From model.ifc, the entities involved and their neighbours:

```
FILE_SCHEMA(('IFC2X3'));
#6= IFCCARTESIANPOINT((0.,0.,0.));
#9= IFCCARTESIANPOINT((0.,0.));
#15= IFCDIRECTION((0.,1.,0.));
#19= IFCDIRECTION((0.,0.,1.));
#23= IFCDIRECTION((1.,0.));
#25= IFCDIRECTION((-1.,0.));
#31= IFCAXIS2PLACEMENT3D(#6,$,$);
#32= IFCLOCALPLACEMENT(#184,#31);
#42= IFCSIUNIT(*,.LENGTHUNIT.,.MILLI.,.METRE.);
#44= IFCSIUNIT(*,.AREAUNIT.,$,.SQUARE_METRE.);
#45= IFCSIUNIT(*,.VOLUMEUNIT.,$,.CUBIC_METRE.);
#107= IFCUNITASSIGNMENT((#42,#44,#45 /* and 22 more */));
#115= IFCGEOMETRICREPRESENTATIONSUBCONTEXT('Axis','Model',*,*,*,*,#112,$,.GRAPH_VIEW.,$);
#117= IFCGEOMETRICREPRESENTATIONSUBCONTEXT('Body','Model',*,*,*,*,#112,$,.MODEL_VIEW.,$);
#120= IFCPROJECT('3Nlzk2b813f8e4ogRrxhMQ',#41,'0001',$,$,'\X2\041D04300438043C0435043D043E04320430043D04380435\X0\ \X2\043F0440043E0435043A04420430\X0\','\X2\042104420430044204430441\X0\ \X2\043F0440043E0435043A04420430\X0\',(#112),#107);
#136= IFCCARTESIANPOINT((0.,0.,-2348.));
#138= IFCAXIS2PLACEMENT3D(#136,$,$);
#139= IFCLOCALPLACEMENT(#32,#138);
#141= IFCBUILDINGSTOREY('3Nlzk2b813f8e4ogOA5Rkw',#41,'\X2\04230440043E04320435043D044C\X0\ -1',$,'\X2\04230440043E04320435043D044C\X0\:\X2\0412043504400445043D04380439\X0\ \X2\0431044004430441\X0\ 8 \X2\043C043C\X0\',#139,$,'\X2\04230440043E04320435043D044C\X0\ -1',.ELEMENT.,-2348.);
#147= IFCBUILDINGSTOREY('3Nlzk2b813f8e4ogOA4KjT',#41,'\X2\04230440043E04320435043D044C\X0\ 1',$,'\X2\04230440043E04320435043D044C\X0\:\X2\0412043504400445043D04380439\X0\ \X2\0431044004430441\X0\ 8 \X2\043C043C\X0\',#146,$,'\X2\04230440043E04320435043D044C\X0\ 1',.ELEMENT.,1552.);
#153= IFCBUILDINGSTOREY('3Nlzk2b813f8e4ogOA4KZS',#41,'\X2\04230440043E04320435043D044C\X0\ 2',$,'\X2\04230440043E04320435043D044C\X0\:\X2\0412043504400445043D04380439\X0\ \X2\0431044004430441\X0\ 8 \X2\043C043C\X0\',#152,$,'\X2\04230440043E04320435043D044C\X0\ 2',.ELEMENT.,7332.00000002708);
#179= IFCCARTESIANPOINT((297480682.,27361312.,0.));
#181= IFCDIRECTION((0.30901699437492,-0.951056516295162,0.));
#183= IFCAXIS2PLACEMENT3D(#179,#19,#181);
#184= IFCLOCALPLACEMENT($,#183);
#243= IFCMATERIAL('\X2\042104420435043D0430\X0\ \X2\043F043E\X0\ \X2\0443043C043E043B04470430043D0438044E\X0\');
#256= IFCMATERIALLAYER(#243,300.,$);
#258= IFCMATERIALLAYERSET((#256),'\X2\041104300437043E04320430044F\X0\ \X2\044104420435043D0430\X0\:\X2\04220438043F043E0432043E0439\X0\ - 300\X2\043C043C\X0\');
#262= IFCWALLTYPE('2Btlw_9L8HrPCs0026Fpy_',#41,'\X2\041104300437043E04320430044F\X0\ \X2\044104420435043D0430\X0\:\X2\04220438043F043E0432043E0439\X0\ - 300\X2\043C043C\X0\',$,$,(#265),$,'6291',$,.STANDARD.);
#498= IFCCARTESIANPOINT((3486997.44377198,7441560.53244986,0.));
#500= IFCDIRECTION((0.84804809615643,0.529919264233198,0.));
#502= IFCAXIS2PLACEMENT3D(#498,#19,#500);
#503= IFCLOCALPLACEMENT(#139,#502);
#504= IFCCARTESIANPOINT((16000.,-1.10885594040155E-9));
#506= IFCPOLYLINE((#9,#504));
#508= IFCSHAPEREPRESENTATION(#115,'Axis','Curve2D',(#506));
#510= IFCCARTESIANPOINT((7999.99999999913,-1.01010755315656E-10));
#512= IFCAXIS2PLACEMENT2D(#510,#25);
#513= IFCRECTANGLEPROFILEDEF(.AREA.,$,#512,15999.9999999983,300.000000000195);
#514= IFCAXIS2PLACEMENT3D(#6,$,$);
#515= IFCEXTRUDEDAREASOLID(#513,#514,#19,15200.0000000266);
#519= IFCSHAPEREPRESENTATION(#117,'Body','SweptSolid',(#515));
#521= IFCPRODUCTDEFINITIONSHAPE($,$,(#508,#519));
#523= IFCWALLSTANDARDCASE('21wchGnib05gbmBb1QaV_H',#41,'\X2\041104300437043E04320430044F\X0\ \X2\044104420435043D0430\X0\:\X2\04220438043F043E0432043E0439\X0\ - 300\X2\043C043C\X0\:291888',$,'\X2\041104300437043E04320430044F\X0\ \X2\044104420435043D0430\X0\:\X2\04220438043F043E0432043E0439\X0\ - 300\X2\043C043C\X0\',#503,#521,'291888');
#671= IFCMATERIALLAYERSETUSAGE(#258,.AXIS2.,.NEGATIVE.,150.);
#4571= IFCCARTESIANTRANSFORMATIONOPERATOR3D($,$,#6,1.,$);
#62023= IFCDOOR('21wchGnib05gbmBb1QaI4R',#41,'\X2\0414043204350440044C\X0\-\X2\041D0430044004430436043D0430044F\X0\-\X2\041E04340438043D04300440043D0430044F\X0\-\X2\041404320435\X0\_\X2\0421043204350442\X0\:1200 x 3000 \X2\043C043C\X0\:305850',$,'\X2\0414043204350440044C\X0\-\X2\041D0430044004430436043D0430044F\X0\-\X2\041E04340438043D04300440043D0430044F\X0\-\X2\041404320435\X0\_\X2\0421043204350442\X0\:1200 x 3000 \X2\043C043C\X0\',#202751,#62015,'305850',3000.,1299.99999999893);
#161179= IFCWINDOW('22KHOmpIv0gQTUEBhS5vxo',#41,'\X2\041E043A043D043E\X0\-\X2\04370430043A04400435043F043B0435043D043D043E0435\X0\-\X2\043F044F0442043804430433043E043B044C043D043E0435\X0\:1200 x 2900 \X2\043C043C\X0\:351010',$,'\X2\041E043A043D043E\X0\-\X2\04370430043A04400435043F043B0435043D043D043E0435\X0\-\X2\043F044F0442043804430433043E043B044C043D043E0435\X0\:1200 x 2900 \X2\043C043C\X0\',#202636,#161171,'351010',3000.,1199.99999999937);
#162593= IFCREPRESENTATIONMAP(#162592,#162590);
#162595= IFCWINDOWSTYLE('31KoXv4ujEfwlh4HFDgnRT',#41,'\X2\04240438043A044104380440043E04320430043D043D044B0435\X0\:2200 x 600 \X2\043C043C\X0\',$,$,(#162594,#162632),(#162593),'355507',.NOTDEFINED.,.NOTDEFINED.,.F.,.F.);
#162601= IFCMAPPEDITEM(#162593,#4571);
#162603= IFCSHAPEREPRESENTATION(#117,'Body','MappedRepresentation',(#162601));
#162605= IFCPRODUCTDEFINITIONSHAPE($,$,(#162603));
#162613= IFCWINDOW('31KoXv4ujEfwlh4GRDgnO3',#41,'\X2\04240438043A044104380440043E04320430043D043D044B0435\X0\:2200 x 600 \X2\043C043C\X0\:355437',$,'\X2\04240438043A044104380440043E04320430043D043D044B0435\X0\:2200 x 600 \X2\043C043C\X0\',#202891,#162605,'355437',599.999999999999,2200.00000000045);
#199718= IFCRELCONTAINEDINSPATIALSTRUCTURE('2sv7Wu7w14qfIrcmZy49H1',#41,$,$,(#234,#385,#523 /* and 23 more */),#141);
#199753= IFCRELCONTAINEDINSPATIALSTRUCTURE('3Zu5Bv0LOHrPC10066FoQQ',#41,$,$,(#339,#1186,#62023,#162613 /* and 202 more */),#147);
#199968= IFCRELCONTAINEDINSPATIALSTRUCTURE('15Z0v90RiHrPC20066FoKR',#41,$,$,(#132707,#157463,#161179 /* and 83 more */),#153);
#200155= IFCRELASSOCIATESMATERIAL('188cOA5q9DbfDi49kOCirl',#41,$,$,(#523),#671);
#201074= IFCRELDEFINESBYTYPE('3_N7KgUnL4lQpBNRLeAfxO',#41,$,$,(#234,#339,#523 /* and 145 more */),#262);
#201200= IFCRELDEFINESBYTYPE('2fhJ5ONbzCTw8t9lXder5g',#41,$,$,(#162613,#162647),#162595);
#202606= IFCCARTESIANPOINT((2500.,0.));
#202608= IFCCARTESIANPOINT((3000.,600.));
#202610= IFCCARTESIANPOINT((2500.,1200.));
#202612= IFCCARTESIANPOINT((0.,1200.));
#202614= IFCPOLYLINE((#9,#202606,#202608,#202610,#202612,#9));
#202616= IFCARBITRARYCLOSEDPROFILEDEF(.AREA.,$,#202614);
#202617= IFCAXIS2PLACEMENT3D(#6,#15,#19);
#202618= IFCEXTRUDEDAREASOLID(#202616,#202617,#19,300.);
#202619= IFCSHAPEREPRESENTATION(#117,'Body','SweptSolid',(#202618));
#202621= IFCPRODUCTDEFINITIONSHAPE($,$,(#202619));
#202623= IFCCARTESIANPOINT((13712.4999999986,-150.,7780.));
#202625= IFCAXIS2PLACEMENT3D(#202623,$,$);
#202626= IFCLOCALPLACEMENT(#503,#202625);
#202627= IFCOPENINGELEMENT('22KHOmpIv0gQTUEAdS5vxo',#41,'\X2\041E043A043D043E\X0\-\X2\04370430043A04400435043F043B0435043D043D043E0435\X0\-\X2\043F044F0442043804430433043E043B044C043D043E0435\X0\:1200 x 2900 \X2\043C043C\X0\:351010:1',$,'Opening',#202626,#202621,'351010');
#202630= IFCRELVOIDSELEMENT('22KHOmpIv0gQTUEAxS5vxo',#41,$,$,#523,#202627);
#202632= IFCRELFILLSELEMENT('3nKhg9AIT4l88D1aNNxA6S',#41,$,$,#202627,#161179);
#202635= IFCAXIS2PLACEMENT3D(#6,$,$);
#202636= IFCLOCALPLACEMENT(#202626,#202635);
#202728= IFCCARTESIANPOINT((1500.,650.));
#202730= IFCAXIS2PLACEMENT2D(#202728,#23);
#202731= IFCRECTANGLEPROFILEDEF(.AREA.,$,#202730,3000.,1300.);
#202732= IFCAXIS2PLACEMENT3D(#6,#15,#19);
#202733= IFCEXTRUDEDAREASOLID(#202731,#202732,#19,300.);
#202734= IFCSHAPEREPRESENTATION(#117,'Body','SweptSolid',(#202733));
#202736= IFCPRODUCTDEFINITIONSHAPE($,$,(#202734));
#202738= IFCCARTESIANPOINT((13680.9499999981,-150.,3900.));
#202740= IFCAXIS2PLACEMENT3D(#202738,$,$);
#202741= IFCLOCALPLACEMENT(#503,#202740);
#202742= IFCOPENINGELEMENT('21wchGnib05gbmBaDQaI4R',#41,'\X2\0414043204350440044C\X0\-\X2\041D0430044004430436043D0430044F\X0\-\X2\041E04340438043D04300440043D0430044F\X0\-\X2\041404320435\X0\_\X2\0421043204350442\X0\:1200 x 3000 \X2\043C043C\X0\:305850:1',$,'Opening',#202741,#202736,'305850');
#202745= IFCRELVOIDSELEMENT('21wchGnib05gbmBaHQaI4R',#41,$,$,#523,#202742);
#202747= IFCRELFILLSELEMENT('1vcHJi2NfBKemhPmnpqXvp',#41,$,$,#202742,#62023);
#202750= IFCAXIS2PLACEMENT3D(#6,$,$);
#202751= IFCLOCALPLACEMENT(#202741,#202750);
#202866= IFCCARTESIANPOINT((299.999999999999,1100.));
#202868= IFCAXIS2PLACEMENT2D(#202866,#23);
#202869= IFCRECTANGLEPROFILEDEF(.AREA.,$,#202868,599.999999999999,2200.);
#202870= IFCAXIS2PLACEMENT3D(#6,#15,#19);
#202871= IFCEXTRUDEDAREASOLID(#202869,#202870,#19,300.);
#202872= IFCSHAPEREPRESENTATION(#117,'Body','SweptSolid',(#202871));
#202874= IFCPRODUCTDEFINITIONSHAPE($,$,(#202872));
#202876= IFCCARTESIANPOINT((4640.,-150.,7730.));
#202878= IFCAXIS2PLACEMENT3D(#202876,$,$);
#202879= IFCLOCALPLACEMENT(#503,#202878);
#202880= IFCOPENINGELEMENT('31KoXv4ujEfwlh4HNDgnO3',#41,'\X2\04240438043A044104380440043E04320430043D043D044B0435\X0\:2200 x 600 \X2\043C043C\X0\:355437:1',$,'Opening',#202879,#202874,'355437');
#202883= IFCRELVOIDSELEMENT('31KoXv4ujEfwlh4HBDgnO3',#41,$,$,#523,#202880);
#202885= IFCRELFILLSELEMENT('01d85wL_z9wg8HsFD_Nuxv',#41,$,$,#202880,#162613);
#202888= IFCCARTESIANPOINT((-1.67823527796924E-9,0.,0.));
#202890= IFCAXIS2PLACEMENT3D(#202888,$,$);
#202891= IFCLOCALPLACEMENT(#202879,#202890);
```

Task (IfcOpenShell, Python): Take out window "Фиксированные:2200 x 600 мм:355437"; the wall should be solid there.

```python
import ifcopenshell
import ifcopenshell.api.feature
import ifcopenshell.api.root
import ifcopenshell.geom
import ifcopenshell.util.shape

model = ifcopenshell.open("model.ifc")
settings = ifcopenshell.geom.settings()


def volume(element):
    """Net volume in cubic metres, openings subtracted."""
    shape = ifcopenshell.geom.create_shape(settings, element)
    return ifcopenshell.util.shape.get_volume(shape.geometry)


window = model.by_id(162613)
opening = window.FillsVoids[0].RelatingOpeningElement
wall = opening.VoidsElements[0].RelatingBuildingElement
before = volume(wall)

ifcopenshell.api.root.remove_product(model, product=window)
ifcopenshell.api.feature.remove_feature(model, feature=opening)

after = volume(wall)

print(f"wall volume {before:.3f} -> {after:.3f} m3")

model.write("model_edited.ifc")
```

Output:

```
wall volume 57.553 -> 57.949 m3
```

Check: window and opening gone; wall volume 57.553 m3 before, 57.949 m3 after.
